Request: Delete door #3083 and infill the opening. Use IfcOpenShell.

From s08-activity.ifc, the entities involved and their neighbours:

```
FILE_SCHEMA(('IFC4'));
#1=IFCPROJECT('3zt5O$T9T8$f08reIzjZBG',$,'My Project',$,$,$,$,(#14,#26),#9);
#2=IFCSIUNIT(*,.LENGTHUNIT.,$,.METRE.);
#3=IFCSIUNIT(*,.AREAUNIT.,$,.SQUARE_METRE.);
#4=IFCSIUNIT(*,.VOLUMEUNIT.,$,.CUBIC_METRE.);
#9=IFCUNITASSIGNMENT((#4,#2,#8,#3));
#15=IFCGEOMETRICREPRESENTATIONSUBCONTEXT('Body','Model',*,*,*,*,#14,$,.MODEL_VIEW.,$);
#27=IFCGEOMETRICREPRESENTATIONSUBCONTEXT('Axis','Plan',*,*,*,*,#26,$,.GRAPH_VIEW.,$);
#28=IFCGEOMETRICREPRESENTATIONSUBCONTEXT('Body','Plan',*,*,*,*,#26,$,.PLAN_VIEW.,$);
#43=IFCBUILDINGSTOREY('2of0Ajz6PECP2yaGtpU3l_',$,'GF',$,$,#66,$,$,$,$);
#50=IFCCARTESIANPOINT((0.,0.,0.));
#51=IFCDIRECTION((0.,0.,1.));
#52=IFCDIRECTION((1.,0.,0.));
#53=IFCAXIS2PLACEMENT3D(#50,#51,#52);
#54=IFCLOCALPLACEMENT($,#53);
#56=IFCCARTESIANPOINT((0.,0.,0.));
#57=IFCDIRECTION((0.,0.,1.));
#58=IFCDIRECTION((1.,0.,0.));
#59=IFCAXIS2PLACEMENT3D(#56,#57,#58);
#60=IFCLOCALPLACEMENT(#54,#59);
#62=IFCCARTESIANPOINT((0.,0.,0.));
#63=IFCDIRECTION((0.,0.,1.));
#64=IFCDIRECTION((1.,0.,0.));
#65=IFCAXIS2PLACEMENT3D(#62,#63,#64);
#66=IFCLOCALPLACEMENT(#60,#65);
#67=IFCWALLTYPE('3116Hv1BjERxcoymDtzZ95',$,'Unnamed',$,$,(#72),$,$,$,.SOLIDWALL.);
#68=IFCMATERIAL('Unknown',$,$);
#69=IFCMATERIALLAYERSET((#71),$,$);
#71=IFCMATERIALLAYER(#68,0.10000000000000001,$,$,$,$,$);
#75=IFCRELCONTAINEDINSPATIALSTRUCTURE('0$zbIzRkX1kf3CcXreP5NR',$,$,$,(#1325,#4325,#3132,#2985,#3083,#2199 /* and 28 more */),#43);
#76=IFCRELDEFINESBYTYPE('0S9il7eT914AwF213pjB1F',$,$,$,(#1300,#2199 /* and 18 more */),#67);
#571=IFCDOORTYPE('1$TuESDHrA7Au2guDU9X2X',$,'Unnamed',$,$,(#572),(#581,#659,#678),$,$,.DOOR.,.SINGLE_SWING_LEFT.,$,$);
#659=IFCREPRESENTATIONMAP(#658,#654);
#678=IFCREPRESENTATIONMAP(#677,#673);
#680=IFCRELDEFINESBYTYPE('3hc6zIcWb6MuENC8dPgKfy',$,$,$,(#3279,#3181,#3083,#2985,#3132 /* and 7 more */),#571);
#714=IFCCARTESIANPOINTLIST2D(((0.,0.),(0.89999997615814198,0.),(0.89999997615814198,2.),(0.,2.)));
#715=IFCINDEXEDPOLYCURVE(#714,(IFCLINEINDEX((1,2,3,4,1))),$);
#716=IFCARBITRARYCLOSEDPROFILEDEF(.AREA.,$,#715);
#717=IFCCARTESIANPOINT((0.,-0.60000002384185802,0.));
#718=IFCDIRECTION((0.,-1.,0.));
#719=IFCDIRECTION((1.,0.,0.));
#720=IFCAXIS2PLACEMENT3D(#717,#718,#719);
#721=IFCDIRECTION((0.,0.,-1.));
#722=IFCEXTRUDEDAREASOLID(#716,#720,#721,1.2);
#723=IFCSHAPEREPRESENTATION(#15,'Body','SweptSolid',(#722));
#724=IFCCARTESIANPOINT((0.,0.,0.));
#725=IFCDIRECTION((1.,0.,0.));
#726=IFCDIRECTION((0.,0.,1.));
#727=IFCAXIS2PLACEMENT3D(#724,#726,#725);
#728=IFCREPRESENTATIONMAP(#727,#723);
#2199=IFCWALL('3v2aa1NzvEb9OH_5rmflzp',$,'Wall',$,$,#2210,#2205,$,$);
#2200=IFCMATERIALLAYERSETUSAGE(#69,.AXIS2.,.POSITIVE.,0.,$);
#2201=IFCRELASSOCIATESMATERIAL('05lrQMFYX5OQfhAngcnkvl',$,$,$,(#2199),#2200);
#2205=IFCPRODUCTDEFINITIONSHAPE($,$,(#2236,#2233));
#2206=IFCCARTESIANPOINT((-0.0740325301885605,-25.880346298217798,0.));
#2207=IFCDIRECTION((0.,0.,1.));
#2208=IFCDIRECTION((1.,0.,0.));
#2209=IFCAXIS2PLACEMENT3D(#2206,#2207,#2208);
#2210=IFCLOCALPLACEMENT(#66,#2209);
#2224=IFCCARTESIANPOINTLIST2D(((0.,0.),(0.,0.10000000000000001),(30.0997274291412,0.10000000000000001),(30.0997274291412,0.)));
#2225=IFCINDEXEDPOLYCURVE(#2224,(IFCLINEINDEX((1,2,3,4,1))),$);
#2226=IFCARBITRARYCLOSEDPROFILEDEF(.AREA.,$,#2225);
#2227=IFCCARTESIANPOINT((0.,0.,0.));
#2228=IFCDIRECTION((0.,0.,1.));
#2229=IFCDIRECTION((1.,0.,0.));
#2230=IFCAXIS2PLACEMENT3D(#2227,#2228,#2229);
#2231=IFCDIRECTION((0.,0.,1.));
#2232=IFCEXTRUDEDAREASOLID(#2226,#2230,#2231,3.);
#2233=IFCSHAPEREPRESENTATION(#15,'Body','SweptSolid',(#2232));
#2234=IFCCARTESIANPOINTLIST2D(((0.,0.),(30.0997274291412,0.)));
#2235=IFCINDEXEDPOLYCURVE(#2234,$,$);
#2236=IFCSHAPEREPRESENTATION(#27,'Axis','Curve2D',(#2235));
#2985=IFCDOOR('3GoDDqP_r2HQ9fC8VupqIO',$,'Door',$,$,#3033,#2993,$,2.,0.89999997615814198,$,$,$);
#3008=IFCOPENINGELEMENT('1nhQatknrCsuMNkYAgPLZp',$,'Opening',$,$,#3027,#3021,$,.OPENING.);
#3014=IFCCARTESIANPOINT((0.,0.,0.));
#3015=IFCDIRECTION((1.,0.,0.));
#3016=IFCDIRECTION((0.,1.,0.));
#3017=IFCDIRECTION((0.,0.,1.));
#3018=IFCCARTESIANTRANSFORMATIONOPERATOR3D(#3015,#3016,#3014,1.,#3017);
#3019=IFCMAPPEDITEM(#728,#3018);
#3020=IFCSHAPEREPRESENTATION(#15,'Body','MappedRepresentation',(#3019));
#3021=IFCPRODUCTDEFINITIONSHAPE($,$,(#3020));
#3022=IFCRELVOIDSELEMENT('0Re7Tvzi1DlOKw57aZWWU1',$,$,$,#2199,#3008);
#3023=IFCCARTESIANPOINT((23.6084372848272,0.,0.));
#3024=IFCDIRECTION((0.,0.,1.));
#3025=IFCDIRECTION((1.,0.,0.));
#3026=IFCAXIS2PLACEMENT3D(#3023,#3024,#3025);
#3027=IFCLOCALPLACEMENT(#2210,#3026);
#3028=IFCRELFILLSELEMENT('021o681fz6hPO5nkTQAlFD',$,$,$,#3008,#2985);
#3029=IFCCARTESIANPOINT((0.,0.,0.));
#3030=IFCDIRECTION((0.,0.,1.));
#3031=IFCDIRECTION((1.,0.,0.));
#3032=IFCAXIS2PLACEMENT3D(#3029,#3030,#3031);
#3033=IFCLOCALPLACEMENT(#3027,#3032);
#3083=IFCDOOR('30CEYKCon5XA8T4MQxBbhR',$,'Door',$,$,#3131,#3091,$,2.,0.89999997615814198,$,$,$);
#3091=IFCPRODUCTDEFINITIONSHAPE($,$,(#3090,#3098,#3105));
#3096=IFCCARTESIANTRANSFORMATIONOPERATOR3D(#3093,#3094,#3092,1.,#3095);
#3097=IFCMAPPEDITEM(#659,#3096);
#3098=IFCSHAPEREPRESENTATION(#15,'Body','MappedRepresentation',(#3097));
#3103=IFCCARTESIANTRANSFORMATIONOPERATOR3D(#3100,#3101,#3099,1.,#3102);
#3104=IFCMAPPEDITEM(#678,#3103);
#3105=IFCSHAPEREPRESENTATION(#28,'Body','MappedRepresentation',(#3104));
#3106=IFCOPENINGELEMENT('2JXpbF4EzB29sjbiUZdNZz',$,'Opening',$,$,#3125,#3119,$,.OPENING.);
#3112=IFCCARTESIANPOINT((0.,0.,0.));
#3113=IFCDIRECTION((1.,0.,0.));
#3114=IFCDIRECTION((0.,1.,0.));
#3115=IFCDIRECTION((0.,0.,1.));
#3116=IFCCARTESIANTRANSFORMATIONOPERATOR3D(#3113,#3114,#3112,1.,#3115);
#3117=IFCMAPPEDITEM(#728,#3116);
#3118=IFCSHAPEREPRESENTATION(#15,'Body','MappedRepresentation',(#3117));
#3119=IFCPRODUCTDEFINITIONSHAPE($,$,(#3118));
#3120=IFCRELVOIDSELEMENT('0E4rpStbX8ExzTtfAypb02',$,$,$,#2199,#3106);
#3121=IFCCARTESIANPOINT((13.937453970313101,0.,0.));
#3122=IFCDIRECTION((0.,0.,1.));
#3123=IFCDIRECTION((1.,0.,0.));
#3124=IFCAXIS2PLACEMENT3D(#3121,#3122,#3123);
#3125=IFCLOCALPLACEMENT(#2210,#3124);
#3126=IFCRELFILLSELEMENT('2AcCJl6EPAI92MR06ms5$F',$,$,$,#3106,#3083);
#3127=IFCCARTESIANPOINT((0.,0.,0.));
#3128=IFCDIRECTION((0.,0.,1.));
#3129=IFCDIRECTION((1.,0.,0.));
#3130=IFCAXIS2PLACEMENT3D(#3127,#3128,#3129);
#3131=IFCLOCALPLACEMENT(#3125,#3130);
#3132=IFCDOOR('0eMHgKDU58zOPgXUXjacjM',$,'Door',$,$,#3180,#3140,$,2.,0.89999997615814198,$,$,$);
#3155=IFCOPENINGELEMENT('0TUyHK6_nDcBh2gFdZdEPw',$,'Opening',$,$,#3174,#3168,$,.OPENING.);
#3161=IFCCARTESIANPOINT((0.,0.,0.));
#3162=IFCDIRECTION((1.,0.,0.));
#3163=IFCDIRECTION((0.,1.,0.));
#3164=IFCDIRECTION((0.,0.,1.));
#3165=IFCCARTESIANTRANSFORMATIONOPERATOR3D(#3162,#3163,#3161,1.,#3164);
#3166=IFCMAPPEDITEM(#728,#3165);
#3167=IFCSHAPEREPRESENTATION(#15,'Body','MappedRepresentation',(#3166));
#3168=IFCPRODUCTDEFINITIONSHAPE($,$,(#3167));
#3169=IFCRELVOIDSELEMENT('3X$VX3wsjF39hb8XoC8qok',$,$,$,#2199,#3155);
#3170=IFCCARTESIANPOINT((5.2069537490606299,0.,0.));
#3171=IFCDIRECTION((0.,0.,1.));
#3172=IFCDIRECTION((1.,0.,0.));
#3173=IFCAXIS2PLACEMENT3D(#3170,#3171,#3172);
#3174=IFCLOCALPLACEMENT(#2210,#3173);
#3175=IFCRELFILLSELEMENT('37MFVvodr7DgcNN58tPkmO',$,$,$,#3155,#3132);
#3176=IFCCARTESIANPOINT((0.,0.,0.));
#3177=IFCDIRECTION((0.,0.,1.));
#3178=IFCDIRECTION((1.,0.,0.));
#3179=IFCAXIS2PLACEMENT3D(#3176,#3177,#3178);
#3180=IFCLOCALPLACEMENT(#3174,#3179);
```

```python
import ifcopenshell
import ifcopenshell.api.feature
import ifcopenshell.api.root
import ifcopenshell.geom
import ifcopenshell.util.shape

model = ifcopenshell.open("s08-activity.ifc")
settings = ifcopenshell.geom.settings()


def volume(element):
    """Net volume in cubic metres, openings subtracted."""
    shape = ifcopenshell.geom.create_shape(settings, element)
    return ifcopenshell.util.shape.get_volume(shape.geometry)


door = model.by_id(3083)
opening = door.FillsVoids[0].RelatingOpeningElement
wall = opening.VoidsElements[0].RelatingBuildingElement
before = volume(wall)

ifcopenshell.api.root.remove_product(model, product=door)
ifcopenshell.api.feature.remove_feature(model, feature=opening)

after = volume(wall)

print(f"wall volume {before:.3f} -> {after:.3f} m3")

model.write("s08-activity_edited.ifc")
```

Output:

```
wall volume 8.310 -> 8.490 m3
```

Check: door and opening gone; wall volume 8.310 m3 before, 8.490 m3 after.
